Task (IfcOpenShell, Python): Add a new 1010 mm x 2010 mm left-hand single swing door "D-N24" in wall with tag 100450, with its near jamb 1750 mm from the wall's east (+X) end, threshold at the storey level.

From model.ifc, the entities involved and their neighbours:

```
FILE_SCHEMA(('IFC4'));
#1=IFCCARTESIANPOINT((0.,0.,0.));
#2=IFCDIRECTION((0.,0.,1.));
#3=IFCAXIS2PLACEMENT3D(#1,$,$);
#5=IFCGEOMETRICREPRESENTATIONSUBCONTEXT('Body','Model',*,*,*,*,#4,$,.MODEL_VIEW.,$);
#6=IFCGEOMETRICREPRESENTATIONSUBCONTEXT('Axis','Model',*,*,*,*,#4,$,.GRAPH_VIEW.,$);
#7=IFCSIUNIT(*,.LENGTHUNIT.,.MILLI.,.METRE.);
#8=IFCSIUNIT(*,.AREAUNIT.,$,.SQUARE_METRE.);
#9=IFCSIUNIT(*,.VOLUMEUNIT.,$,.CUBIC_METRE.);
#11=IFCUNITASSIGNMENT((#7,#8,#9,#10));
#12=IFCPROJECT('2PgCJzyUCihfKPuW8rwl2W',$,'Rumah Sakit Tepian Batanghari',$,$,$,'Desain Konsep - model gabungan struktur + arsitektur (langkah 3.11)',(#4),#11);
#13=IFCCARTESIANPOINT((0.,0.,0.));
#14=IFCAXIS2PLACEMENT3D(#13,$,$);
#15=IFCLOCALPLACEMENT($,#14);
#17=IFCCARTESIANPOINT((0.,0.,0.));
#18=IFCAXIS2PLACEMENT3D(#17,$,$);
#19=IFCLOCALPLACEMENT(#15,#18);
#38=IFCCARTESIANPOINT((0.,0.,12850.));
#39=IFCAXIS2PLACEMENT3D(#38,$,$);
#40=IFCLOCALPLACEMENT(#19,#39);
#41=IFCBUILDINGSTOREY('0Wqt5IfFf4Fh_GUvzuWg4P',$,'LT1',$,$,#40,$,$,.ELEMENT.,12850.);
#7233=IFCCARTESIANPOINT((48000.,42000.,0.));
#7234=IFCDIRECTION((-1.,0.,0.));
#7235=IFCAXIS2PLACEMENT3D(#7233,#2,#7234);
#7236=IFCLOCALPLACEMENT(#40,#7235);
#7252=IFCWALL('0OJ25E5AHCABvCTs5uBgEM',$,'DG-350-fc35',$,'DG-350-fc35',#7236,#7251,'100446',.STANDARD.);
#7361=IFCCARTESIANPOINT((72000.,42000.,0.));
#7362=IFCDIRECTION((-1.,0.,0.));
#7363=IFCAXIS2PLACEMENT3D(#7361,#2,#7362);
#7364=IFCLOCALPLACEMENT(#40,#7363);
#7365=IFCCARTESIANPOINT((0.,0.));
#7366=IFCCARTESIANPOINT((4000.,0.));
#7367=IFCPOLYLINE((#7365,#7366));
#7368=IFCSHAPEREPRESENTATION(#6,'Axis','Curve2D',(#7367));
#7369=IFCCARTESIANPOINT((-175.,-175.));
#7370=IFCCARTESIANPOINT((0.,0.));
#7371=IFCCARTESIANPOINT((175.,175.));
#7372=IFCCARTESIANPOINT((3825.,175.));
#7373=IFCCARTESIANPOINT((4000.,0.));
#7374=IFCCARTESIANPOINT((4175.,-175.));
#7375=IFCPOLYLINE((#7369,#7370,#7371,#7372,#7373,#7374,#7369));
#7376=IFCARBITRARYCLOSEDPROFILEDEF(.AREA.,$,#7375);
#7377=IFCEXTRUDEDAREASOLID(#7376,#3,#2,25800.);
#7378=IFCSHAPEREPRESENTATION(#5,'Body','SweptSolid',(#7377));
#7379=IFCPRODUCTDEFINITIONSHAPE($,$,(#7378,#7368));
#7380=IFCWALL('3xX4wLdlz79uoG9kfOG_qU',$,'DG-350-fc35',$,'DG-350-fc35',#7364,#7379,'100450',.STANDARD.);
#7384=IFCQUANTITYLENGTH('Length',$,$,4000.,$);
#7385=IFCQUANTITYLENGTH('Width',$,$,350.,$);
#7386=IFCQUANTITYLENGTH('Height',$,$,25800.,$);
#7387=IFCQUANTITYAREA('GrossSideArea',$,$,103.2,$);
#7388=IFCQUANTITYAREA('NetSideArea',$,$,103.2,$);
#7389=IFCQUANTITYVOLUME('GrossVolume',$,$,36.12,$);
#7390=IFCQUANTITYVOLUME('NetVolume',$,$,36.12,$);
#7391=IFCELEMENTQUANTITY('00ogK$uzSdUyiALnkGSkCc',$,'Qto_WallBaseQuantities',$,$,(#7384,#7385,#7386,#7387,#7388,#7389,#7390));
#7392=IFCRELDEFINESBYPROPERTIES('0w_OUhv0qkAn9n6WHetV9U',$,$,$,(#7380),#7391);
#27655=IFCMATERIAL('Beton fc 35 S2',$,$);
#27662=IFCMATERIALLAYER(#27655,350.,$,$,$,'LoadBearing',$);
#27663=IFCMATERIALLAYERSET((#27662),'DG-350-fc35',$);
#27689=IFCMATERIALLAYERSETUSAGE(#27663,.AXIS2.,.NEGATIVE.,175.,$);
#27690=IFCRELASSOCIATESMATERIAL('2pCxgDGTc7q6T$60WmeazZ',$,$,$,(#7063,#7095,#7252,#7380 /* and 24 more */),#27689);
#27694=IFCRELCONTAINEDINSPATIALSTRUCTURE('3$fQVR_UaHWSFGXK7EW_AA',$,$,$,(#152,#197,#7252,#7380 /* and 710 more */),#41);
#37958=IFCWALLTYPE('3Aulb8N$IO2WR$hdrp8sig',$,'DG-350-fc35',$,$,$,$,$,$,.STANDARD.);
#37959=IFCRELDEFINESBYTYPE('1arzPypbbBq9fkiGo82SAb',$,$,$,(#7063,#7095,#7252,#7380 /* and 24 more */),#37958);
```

```python
import numpy as np
import ifcopenshell
import ifcopenshell.api.feature
import ifcopenshell.api.geometry
import ifcopenshell.api.pset
import ifcopenshell.api.root
import ifcopenshell.api.spatial
import ifcopenshell.geom
import ifcopenshell.util.element
import ifcopenshell.util.placement
import ifcopenshell.util.representation
import ifcopenshell.util.shape
import ifcopenshell.util.unit

model = ifcopenshell.open("model.ifc")
unit_scale = ifcopenshell.util.unit.calculate_unit_scale(model)
area_scale = ifcopenshell.util.unit.calculate_unit_scale(model, "AREAUNIT")
volume_scale = ifcopenshell.util.unit.calculate_unit_scale(model, "VOLUMEUNIT")
settings = ifcopenshell.geom.settings()


def volume(element):
    """Net volume in cubic metres, openings subtracted."""
    shape = ifcopenshell.geom.create_shape(settings, element)
    return ifcopenshell.util.shape.get_volume(shape.geometry)


wall = model.by_guid("3xX4wLdlz79uoG9kfOG_qU")
storey = ifcopenshell.util.element.get_container(wall, ifc_class="IfcBuildingStorey")
context = ifcopenshell.util.representation.get_context(model, "Model", "Body", "MODEL_VIEW")
before = volume(wall)

width, height, from_end, sill = 1.01, 2.01, 1.75, 0.0  # metres

# The wall runs along its own X axis, and the end named is its -X end.
wall_shape = ifcopenshell.geom.create_shape(settings, wall)
x, y, z = ifcopenshell.util.shape.get_vertices(wall_shape.geometry).T
start = x.min() + from_end
face, thickness = float(y.min()), float(y.max() - y.min())
wall_matrix = ifcopenshell.util.placement.get_local_placement(wall.ObjectPlacement)
level = ifcopenshell.util.placement.get_local_placement(storey.ObjectPlacement)[2, 3]


def in_wall(x, y):
    """Placement at x, y metres in the wall's axes, at sill height."""
    matrix = wall_matrix.copy()
    matrix[:, 3] = wall_matrix @ np.array([x / unit_scale, y / unit_scale, 0.0, 1.0])
    matrix[2, 3] = level + sill / unit_scale
    return matrix


# Opening: a box that overshoots both wall faces by 50 mm.
opening = ifcopenshell.api.root.create_entity(model, ifc_class="IfcOpeningElement", predefined_type="OPENING")
box = ifcopenshell.api.geometry.add_wall_representation(
    model, context=context, length=width, height=height, thickness=thickness + 0.1
)
ifcopenshell.api.geometry.assign_representation(model, product=opening, representation=box)
ifcopenshell.api.geometry.edit_object_placement(model, product=opening, matrix=in_wall(start, face - 0.05), is_si=False)
ifcopenshell.api.feature.add_feature(model, feature=opening, element=wall)

door = ifcopenshell.api.root.create_entity(model, ifc_class="IfcDoor", name="D-N24", predefined_type="DOOR")
door.OverallWidth, door.OverallHeight = width / unit_scale, height / unit_scale
door.OperationType = "SINGLE_SWING_LEFT"
body = ifcopenshell.api.geometry.add_door_representation(
    model,
    context=context,
    overall_width=door.OverallWidth,
    overall_height=door.OverallHeight,
    operation_type="SINGLE_SWING_LEFT",
    lining_properties={"LiningDepth": thickness / unit_scale, "ThresholdDepth": thickness / unit_scale},
)
ifcopenshell.api.geometry.assign_representation(model, product=door, representation=body)
ifcopenshell.api.spatial.assign_container(model, products=[door], relating_structure=storey)
ifcopenshell.api.feature.add_filling(model, opening=opening, element=door)

# The lining spans the wall, so the door starts at the wall face.
ifcopenshell.api.geometry.edit_object_placement(model, product=door, matrix=in_wall(start, face), is_si=False)

after = volume(wall)

# Update the wall's stored quantities.
qto = model.by_id(ifcopenshell.util.element.get_pset(wall, "Qto_WallBaseQuantities", should_inherit=False)["id"])
ifcopenshell.api.pset.edit_qto(model, qto=qto, properties={
    "NetSideArea": after / thickness / area_scale,
    "NetVolume": after / volume_scale,
})

print(f"wall volume {before:.3f} -> {after:.3f} m3")

model.write("model_rev.ifc")
```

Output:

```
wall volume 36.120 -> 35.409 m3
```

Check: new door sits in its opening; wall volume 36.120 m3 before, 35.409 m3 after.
